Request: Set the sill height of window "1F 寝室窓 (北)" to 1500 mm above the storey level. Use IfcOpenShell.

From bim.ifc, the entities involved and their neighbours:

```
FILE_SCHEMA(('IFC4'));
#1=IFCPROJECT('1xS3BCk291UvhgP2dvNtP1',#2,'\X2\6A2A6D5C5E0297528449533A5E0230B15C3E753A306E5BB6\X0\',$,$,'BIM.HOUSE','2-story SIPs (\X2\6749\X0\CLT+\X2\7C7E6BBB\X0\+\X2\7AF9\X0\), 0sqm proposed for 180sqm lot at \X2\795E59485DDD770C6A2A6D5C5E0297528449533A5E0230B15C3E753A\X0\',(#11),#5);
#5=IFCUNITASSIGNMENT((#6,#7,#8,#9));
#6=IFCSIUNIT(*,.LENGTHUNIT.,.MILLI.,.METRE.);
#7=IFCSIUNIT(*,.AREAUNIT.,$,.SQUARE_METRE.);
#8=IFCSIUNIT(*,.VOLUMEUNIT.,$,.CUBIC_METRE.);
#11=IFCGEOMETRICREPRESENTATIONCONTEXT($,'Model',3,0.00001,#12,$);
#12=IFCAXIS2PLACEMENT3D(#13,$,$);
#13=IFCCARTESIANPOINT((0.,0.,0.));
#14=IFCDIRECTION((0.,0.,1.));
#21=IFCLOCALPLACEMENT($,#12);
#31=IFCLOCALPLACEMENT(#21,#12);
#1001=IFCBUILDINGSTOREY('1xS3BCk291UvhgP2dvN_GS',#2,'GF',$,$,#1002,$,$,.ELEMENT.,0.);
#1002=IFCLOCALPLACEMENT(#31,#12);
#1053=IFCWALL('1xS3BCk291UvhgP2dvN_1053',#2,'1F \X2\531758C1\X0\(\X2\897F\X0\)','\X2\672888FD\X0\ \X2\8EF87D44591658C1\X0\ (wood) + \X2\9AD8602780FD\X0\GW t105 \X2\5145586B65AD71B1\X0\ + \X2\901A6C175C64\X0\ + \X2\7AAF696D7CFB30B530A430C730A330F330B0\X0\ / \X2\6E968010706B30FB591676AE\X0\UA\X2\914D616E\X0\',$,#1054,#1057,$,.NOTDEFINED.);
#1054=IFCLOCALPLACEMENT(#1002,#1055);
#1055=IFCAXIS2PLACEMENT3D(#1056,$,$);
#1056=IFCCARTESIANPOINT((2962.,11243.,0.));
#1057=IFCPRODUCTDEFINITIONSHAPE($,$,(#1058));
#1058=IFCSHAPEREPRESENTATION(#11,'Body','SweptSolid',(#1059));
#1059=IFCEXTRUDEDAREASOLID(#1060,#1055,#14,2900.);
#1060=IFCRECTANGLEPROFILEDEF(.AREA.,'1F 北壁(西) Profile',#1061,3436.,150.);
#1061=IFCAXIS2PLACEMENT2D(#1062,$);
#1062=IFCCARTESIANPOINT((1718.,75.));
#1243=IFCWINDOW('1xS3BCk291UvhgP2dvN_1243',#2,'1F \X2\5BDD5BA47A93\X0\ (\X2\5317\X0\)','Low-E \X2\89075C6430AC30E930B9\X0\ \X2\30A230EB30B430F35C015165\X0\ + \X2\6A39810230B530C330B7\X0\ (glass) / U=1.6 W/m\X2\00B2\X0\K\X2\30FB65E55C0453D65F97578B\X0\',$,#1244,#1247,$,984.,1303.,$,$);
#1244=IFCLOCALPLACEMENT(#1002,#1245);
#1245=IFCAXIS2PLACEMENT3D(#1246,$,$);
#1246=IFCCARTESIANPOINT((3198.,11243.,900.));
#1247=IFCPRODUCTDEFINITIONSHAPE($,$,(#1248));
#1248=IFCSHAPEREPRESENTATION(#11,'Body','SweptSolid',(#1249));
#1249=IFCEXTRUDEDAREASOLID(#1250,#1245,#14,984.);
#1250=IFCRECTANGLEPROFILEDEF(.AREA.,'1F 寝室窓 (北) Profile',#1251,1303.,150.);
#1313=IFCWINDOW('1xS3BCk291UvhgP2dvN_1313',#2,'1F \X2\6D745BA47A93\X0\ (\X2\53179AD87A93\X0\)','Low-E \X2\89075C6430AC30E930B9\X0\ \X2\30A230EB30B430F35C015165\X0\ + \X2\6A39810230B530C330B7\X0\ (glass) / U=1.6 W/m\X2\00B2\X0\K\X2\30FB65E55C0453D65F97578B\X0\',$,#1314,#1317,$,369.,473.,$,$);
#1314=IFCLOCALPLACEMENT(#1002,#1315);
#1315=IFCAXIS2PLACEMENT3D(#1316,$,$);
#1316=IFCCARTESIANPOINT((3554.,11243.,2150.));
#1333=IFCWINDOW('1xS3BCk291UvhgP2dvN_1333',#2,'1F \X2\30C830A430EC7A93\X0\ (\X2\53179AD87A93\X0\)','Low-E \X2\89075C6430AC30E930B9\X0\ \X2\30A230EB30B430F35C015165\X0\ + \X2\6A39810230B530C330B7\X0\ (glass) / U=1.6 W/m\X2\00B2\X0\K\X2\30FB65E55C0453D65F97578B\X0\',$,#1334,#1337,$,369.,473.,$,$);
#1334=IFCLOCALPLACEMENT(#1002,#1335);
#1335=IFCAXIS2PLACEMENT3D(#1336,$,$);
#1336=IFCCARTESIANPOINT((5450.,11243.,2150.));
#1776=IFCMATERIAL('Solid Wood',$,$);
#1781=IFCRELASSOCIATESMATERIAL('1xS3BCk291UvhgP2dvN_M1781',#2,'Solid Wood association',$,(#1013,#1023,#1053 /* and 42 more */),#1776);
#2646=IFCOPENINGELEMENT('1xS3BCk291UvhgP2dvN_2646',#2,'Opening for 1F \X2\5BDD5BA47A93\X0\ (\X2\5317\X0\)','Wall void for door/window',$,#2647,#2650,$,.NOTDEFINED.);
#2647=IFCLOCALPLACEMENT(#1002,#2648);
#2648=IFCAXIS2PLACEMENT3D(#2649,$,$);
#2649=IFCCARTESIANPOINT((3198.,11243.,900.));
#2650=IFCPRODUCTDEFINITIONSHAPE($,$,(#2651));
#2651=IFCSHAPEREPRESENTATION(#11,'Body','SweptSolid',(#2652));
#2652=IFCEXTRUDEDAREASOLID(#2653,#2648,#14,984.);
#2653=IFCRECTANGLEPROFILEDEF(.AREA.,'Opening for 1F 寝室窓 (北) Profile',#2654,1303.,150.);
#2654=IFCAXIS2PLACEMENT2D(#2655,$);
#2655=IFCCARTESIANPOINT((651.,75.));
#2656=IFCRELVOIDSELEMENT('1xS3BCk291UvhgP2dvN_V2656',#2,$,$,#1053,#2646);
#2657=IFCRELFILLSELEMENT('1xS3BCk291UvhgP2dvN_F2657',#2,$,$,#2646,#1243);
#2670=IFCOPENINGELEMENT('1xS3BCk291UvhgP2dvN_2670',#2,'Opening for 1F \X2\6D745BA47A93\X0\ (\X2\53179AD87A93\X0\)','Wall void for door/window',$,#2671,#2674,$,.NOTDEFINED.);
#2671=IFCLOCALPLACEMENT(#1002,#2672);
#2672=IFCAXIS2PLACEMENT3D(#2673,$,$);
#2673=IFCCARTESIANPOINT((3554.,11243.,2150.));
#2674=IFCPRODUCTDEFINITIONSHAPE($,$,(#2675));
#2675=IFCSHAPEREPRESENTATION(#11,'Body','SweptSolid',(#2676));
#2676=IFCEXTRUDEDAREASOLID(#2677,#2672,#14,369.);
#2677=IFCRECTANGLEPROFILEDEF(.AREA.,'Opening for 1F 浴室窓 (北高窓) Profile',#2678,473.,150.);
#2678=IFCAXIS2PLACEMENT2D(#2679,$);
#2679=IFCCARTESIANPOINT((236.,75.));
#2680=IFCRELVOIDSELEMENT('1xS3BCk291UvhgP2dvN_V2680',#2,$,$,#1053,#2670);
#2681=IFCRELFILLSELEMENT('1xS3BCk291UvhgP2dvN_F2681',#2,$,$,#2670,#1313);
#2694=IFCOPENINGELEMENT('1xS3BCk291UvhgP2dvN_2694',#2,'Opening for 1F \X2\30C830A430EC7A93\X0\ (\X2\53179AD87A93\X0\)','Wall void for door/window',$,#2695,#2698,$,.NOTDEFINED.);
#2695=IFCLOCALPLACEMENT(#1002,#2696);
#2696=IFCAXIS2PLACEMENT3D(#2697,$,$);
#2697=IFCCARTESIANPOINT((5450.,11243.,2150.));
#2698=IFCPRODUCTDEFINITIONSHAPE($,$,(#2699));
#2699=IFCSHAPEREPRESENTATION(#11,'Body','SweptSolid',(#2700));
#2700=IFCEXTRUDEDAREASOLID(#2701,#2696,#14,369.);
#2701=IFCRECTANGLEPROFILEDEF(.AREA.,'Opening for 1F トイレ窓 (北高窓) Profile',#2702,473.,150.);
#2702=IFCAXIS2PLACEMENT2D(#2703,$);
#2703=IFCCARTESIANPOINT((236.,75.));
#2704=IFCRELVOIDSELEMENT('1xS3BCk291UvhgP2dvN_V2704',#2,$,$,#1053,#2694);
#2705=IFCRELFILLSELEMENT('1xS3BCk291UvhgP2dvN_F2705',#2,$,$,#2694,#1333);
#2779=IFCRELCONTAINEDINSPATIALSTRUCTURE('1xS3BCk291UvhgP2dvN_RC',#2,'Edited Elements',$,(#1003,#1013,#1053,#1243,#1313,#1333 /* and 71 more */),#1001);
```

```python
import numpy as np
import ifcopenshell
import ifcopenshell.api.geometry
import ifcopenshell.geom
import ifcopenshell.util.element
import ifcopenshell.util.placement
import ifcopenshell.util.shape
import ifcopenshell.util.unit

model = ifcopenshell.open("bim.ifc")
unit_scale = ifcopenshell.util.unit.calculate_unit_scale(model)

window = model.by_guid("1xS3BCk291UvhgP2dvN_1243")
opening = window.FillsVoids[0].RelatingOpeningElement
storey = ifcopenshell.util.element.get_container(window, ifc_class="IfcBuildingStorey")
level = ifcopenshell.util.placement.get_local_placement(storey.ObjectPlacement)[2, 3]

# The opening's origin need not be at the sill, so measure its lowest point.
shape = ifcopenshell.geom.create_shape(ifcopenshell.geom.settings(), opening)
bottom = ifcopenshell.util.shape.get_shape_bottom_elevation(shape, shape.geometry) / unit_scale
dz = level + 1.5 / unit_scale - bottom

shift = np.array([0.0, 0.0, dz])
# The window is not placed relative to its opening, so move both.
for product in (opening, window):
    matrix = ifcopenshell.util.placement.get_local_placement(product.ObjectPlacement)
    matrix[:3, 3] += shift
    ifcopenshell.api.geometry.edit_object_placement(model, product=product, matrix=matrix, is_si=False)

print(f"moved by {dz * unit_scale:+.3f} m")

model.write("bim-out.ifc")
```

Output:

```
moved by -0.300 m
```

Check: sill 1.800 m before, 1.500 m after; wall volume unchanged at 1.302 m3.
